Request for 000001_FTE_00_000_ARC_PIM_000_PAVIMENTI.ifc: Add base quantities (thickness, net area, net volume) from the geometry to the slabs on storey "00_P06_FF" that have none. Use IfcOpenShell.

First a look at what the model holds.

```python
import ifcopenshell
import ifcopenshell.util.element
import ifcopenshell.util.unit

model = ifcopenshell.open("000001_FTE_00_000_ARC_PIM_000_PAVIMENTI.ifc")
print(model.schema)
for unit_type in ("LENGTHUNIT", "AREAUNIT", "VOLUMEUNIT"):
    print(unit_type, ifcopenshell.util.unit.calculate_unit_scale(model, unit_type))
storey = next(s for s in model.by_type("IfcBuildingStorey") if s.Name == "00_P06_FF")
slabs = [e for e in ifcopenshell.util.element.get_decomposition(storey) if e.is_a("IfcSlab")]
for e in sorted(slabs, key=lambda e: e.id()):
    print(e.id(), e.is_a(), e.Name, list(ifcopenshell.util.element.get_psets(e, qtos_only=True)), sep=" | ")
```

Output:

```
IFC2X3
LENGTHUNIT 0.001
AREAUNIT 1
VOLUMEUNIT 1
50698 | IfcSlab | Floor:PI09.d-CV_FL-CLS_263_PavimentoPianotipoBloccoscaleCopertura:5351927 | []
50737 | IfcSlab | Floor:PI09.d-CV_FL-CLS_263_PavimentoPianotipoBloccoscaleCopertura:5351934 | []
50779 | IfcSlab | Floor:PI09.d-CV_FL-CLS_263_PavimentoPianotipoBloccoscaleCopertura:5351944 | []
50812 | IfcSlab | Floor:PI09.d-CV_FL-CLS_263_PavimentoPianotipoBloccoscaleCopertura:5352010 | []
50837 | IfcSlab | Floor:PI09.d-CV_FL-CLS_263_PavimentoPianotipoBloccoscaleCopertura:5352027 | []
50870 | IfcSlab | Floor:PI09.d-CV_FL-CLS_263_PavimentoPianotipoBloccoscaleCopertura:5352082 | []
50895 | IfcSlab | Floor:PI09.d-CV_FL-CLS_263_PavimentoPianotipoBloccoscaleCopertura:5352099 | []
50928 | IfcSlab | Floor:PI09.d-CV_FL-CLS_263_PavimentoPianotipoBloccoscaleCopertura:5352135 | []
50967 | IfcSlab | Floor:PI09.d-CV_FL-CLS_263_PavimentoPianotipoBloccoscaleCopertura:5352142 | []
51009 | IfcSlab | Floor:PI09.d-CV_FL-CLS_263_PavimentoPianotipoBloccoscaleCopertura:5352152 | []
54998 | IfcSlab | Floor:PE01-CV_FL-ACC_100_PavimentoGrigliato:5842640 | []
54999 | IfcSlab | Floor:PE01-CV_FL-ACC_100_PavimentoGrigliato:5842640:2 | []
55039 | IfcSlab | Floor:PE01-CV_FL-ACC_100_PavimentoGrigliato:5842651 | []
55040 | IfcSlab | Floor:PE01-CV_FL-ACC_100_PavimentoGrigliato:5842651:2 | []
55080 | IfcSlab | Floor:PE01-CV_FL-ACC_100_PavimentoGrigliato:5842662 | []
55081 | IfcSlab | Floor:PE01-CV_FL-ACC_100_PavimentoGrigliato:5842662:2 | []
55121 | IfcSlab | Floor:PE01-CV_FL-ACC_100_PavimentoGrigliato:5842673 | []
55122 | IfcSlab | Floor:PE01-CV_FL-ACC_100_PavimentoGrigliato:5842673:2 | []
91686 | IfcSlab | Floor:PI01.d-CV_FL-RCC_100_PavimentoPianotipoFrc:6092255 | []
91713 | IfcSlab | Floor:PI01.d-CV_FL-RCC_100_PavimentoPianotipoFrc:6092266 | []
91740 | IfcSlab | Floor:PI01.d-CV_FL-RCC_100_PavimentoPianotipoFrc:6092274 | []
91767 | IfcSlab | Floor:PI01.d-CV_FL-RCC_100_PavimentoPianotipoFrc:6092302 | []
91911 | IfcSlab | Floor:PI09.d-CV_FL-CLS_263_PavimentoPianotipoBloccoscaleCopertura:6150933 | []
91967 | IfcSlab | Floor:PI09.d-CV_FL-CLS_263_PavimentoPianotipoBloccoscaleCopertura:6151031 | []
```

```python
import ifcopenshell
import ifcopenshell.api.pset
import ifcopenshell.geom
import ifcopenshell.util.element
import ifcopenshell.util.shape
import ifcopenshell.util.unit

model = ifcopenshell.open("000001_FTE_00_000_ARC_PIM_000_PAVIMENTI.ifc")
unit_scale = ifcopenshell.util.unit.calculate_unit_scale(model)
area_scale = ifcopenshell.util.unit.calculate_unit_scale(model, "AREAUNIT")
volume_scale = ifcopenshell.util.unit.calculate_unit_scale(model, "VOLUMEUNIT")
settings = ifcopenshell.geom.settings()

storey = next(s for s in model.by_type("IfcBuildingStorey") if s.Name == "00_P06_FF")
slabs = [e for e in ifcopenshell.util.element.get_decomposition(storey) if e.is_a("IfcSlab")]

for e in sorted(slabs, key=lambda e: e.id()):
    if ifcopenshell.util.element.get_psets(e, qtos_only=True, should_inherit=False):
        continue
    # Geometry comes back in metres, in the element's own axes.
    shape = ifcopenshell.geom.create_shape(settings, e)
    values = {
        "Width": ifcopenshell.util.shape.get_z(shape.geometry) / unit_scale,
        "NetArea": ifcopenshell.util.shape.get_footprint_area(shape.geometry) / area_scale,
        "NetVolume": ifcopenshell.util.shape.get_volume(shape.geometry) / volume_scale,
    }
    qto = ifcopenshell.api.pset.add_qto(model, product=e, name="BaseQuantities")
    ifcopenshell.api.pset.edit_qto(model, qto=qto, properties=values)
    print(e.id(), {k: round(v, 3) for k, v in values.items()})

model.write("000001_FTE_00_000_ARC_PIM_000_PAVIMENTI_v2.ifc")
```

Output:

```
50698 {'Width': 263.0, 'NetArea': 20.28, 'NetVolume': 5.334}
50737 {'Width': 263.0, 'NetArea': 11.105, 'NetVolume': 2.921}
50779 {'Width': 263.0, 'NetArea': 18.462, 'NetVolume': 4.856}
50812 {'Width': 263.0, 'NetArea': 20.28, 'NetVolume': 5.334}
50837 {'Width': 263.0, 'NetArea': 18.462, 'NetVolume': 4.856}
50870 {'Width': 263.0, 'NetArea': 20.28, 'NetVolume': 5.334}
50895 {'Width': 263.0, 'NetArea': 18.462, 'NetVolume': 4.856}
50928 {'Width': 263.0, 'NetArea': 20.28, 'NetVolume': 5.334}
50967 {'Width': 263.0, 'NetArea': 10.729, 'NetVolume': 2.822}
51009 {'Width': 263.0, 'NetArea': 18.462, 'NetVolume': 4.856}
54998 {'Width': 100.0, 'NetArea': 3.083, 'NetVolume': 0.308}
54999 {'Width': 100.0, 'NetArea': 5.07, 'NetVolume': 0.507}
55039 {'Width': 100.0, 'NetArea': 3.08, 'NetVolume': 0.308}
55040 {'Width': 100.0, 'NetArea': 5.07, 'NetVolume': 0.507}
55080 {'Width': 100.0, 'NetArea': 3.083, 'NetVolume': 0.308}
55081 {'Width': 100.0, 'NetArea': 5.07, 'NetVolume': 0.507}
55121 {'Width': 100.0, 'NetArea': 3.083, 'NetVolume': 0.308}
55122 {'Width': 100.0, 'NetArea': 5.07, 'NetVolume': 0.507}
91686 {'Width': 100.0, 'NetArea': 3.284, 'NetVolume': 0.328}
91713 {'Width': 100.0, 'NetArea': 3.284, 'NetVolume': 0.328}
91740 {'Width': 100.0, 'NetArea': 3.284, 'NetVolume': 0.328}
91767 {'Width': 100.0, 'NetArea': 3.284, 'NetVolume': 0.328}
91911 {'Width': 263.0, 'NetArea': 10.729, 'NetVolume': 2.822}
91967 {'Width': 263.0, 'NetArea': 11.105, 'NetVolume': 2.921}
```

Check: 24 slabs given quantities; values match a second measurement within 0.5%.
